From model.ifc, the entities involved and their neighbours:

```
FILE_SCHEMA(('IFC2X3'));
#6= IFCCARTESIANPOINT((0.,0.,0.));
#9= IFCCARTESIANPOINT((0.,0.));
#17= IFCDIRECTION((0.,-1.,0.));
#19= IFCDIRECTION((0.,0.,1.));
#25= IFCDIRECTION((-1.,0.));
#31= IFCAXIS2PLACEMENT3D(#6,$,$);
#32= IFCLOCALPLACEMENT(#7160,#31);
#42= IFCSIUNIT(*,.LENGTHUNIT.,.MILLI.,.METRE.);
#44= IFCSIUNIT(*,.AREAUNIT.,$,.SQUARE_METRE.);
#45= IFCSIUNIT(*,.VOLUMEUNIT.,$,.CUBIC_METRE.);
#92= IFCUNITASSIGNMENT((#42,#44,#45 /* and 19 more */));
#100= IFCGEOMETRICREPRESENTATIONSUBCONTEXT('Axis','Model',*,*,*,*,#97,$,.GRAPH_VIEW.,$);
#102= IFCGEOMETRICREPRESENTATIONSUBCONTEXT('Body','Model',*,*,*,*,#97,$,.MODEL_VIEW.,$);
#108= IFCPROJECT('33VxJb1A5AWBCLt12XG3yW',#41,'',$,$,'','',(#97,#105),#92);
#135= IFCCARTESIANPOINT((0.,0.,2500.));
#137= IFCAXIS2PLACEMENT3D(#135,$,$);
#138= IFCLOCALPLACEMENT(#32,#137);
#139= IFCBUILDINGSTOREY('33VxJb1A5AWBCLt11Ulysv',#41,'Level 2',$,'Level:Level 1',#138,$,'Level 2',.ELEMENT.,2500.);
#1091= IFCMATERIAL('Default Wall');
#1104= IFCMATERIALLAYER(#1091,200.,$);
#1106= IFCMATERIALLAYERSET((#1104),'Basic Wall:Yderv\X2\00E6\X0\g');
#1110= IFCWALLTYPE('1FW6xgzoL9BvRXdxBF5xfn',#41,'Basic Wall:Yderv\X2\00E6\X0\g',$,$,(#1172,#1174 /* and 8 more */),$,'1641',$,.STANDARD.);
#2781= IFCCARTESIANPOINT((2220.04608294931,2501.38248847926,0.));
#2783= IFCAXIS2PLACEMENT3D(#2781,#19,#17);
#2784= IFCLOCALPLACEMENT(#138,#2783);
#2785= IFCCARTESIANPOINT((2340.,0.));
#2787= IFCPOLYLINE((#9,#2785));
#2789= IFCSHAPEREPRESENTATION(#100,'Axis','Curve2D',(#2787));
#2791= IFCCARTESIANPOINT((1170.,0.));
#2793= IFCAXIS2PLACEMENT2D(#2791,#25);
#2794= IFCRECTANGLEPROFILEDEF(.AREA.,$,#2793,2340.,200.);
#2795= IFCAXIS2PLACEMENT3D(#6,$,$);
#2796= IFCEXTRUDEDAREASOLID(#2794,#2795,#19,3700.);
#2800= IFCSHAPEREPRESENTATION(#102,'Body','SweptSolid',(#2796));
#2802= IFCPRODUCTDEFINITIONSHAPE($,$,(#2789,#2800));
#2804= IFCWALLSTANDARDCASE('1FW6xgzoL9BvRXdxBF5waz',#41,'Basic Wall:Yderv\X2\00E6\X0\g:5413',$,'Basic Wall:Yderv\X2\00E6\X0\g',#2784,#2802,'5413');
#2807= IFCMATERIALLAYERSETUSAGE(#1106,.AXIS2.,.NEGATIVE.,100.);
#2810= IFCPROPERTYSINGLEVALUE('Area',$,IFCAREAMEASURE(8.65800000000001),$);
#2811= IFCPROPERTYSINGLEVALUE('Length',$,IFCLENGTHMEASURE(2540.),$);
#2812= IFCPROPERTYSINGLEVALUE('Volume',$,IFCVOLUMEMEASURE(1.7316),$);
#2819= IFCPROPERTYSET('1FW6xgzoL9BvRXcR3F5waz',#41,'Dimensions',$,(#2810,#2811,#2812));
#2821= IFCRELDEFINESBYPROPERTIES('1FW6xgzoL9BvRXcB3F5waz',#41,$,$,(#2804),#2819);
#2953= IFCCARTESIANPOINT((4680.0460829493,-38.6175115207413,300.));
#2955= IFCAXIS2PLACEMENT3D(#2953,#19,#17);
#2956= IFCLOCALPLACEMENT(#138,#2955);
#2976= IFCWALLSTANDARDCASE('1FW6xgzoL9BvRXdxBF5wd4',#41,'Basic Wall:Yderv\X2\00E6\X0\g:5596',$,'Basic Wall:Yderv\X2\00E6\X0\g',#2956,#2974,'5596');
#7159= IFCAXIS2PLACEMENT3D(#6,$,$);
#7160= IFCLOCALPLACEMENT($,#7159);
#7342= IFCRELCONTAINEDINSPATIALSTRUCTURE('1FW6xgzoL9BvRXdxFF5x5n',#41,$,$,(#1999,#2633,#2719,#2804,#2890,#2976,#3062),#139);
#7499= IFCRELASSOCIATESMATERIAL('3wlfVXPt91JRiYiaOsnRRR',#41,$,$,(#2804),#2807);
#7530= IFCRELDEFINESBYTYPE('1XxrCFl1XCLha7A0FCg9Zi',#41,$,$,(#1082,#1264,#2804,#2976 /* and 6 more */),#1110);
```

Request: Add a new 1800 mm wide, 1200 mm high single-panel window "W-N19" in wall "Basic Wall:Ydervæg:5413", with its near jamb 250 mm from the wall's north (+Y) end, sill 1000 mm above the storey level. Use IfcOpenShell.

```python
import numpy as np
import ifcopenshell
import ifcopenshell.api.feature
import ifcopenshell.api.geometry
import ifcopenshell.api.pset
import ifcopenshell.api.root
import ifcopenshell.api.spatial
import ifcopenshell.api.type
import ifcopenshell.geom
import ifcopenshell.util.element
import ifcopenshell.util.placement
import ifcopenshell.util.representation
import ifcopenshell.util.shape
import ifcopenshell.util.unit

model = ifcopenshell.open("model.ifc")
unit_scale = ifcopenshell.util.unit.calculate_unit_scale(model)
area_scale = ifcopenshell.util.unit.calculate_unit_scale(model, "AREAUNIT")
volume_scale = ifcopenshell.util.unit.calculate_unit_scale(model, "VOLUMEUNIT")
settings = ifcopenshell.geom.settings()


def volume(element):
    """Net volume in cubic metres, openings subtracted."""
    shape = ifcopenshell.geom.create_shape(settings, element)
    return ifcopenshell.util.shape.get_volume(shape.geometry)


wall = model.by_guid("1FW6xgzoL9BvRXdxBF5waz")
storey = ifcopenshell.util.element.get_container(wall, ifc_class="IfcBuildingStorey")
context = ifcopenshell.util.representation.get_context(model, "Model", "Body", "MODEL_VIEW")
before = volume(wall)

width, height, from_end, sill = 1.8, 1.2, 0.25, 1  # metres

# The wall runs along its own X axis, and the end named is its -X end.
wall_shape = ifcopenshell.geom.create_shape(settings, wall)
x, y, z = ifcopenshell.util.shape.get_vertices(wall_shape.geometry).T
start = x.min() + from_end
face, thickness = float(y.min()), float(y.max() - y.min())
wall_matrix = ifcopenshell.util.placement.get_local_placement(wall.ObjectPlacement)
level = ifcopenshell.util.placement.get_local_placement(storey.ObjectPlacement)[2, 3]


def in_wall(x, y):
    """Placement at x, y metres in the wall's axes, at sill height."""
    matrix = wall_matrix.copy()
    matrix[:, 3] = wall_matrix @ np.array([x / unit_scale, y / unit_scale, 0.0, 1.0])
    matrix[2, 3] = level + sill / unit_scale
    return matrix


# Opening: a box that overshoots both wall faces by 50 mm.
opening = ifcopenshell.api.root.create_entity(model, ifc_class="IfcOpeningElement")
box = ifcopenshell.api.geometry.add_wall_representation(
    model, context=context, length=width, height=height, thickness=thickness + 0.1
)
ifcopenshell.api.geometry.assign_representation(model, product=opening, representation=box)
ifcopenshell.api.geometry.edit_object_placement(model, product=opening, matrix=in_wall(start, face - 0.05), is_si=False)
ifcopenshell.api.feature.add_feature(model, feature=opening, element=wall)

window = ifcopenshell.api.root.create_entity(model, ifc_class="IfcWindow", name="W-N19")
window.OverallWidth, window.OverallHeight = width / unit_scale, height / unit_scale
body = ifcopenshell.api.geometry.add_window_representation(
    model,
    context=context,
    overall_width=window.OverallWidth,
    overall_height=window.OverallHeight,
    partition_type="SINGLE_PANEL",
)
ifcopenshell.api.geometry.assign_representation(model, product=window, representation=body)
ifcopenshell.api.spatial.assign_container(model, products=[window], relating_structure=storey)
fills = ifcopenshell.api.feature.add_filling(model, opening=opening, element=window)
fills.OwnerHistory = window.OwnerHistory  # required in IFC2X3

# IFC2X3 keeps the operation on the window style.
style = ifcopenshell.api.root.create_entity(model, ifc_class="IfcWindowStyle", name="W-N19")
style.OperationType, style.ConstructionType = "SINGLE_PANEL", "NOTDEFINED"
style.ParameterTakesPrecedence = style.Sizeable = False
ifcopenshell.api.type.assign_type(model, related_objects=[window], relating_type=style)

# Centre the window in the wall's thickness.
ifcopenshell.api.geometry.edit_object_placement(model, product=window, matrix=in_wall(start, face), is_si=False)
window_shape = ifcopenshell.geom.create_shape(settings, window)
depth = ifcopenshell.util.shape.get_vertices(window_shape.geometry)[:, 1]
offset = face + thickness / 2 - (depth.min() + depth.max()) / 2
ifcopenshell.api.geometry.edit_object_placement(model, product=window, matrix=in_wall(start, offset), is_si=False)

after = volume(wall)

# Update the wall's stored quantities.
pset = model.by_id(ifcopenshell.util.element.get_pset(wall, "Dimensions", should_inherit=False)["id"])
ifcopenshell.api.pset.edit_pset(model, pset=pset, properties={
    "Area": model.create_entity("IfcAreaMeasure", after / thickness / area_scale),
    "Volume": model.create_entity("IfcVolumeMeasure", after / volume_scale),
})

print(f"wall volume {before:.3f} -> {after:.3f} m3")

model.write("model_v2.ifc")
```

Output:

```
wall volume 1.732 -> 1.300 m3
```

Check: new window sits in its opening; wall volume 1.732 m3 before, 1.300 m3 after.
